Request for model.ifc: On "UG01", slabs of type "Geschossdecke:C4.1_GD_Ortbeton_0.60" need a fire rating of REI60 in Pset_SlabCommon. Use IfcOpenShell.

First a look at what the model holds.

```python
import ifcopenshell
import ifcopenshell.util.element

model = ifcopenshell.open("model.ifc")
print(model.schema)
storey = next(s for s in model.by_type("IfcBuildingStorey") if s.Name == "UG01")
slabs = [e for e in ifcopenshell.util.element.get_decomposition(storey) if e.is_a("IfcSlab")]
seen = {}
for e in slabs:
    element_type = ifcopenshell.util.element.get_type(e)
    key = (element_type.Name if element_type != e and element_type else None, ifcopenshell.util.element.get_pset(e, "Pset_SlabCommon", "FireRating"))
    seen[key] = seen.get(key, 0) + 1
for (name, value), count in sorted(seen.items(), key=str):
    print(count, "x", name, "|", value)
```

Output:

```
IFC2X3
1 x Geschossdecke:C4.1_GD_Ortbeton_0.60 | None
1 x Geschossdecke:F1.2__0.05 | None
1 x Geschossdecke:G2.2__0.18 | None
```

```python
import ifcopenshell
import ifcopenshell.api.pset
import ifcopenshell.util.element

model = ifcopenshell.open("model.ifc")

storey = next(s for s in model.by_type("IfcBuildingStorey") if s.Name == "UG01")
slabs = [e for e in ifcopenshell.util.element.get_decomposition(storey) if e.is_a("IfcSlab")]

count = 0
for e in slabs:
    element_type = ifcopenshell.util.element.get_type(e)
    if element_type in (None, e) or element_type.Name != "Geschossdecke:C4.1_GD_Ortbeton_0.60":
        continue
    # add_pset returns the element's existing set when there is one.
    pset = ifcopenshell.api.pset.add_pset(model, product=e, name="Pset_SlabCommon")
    ifcopenshell.api.pset.edit_pset(model, pset=pset, properties={"FireRating": "REI60"})
    count += 1

print(count, "slabs updated")

model.write("model_updated.ifc")
```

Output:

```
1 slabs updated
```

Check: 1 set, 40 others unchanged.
